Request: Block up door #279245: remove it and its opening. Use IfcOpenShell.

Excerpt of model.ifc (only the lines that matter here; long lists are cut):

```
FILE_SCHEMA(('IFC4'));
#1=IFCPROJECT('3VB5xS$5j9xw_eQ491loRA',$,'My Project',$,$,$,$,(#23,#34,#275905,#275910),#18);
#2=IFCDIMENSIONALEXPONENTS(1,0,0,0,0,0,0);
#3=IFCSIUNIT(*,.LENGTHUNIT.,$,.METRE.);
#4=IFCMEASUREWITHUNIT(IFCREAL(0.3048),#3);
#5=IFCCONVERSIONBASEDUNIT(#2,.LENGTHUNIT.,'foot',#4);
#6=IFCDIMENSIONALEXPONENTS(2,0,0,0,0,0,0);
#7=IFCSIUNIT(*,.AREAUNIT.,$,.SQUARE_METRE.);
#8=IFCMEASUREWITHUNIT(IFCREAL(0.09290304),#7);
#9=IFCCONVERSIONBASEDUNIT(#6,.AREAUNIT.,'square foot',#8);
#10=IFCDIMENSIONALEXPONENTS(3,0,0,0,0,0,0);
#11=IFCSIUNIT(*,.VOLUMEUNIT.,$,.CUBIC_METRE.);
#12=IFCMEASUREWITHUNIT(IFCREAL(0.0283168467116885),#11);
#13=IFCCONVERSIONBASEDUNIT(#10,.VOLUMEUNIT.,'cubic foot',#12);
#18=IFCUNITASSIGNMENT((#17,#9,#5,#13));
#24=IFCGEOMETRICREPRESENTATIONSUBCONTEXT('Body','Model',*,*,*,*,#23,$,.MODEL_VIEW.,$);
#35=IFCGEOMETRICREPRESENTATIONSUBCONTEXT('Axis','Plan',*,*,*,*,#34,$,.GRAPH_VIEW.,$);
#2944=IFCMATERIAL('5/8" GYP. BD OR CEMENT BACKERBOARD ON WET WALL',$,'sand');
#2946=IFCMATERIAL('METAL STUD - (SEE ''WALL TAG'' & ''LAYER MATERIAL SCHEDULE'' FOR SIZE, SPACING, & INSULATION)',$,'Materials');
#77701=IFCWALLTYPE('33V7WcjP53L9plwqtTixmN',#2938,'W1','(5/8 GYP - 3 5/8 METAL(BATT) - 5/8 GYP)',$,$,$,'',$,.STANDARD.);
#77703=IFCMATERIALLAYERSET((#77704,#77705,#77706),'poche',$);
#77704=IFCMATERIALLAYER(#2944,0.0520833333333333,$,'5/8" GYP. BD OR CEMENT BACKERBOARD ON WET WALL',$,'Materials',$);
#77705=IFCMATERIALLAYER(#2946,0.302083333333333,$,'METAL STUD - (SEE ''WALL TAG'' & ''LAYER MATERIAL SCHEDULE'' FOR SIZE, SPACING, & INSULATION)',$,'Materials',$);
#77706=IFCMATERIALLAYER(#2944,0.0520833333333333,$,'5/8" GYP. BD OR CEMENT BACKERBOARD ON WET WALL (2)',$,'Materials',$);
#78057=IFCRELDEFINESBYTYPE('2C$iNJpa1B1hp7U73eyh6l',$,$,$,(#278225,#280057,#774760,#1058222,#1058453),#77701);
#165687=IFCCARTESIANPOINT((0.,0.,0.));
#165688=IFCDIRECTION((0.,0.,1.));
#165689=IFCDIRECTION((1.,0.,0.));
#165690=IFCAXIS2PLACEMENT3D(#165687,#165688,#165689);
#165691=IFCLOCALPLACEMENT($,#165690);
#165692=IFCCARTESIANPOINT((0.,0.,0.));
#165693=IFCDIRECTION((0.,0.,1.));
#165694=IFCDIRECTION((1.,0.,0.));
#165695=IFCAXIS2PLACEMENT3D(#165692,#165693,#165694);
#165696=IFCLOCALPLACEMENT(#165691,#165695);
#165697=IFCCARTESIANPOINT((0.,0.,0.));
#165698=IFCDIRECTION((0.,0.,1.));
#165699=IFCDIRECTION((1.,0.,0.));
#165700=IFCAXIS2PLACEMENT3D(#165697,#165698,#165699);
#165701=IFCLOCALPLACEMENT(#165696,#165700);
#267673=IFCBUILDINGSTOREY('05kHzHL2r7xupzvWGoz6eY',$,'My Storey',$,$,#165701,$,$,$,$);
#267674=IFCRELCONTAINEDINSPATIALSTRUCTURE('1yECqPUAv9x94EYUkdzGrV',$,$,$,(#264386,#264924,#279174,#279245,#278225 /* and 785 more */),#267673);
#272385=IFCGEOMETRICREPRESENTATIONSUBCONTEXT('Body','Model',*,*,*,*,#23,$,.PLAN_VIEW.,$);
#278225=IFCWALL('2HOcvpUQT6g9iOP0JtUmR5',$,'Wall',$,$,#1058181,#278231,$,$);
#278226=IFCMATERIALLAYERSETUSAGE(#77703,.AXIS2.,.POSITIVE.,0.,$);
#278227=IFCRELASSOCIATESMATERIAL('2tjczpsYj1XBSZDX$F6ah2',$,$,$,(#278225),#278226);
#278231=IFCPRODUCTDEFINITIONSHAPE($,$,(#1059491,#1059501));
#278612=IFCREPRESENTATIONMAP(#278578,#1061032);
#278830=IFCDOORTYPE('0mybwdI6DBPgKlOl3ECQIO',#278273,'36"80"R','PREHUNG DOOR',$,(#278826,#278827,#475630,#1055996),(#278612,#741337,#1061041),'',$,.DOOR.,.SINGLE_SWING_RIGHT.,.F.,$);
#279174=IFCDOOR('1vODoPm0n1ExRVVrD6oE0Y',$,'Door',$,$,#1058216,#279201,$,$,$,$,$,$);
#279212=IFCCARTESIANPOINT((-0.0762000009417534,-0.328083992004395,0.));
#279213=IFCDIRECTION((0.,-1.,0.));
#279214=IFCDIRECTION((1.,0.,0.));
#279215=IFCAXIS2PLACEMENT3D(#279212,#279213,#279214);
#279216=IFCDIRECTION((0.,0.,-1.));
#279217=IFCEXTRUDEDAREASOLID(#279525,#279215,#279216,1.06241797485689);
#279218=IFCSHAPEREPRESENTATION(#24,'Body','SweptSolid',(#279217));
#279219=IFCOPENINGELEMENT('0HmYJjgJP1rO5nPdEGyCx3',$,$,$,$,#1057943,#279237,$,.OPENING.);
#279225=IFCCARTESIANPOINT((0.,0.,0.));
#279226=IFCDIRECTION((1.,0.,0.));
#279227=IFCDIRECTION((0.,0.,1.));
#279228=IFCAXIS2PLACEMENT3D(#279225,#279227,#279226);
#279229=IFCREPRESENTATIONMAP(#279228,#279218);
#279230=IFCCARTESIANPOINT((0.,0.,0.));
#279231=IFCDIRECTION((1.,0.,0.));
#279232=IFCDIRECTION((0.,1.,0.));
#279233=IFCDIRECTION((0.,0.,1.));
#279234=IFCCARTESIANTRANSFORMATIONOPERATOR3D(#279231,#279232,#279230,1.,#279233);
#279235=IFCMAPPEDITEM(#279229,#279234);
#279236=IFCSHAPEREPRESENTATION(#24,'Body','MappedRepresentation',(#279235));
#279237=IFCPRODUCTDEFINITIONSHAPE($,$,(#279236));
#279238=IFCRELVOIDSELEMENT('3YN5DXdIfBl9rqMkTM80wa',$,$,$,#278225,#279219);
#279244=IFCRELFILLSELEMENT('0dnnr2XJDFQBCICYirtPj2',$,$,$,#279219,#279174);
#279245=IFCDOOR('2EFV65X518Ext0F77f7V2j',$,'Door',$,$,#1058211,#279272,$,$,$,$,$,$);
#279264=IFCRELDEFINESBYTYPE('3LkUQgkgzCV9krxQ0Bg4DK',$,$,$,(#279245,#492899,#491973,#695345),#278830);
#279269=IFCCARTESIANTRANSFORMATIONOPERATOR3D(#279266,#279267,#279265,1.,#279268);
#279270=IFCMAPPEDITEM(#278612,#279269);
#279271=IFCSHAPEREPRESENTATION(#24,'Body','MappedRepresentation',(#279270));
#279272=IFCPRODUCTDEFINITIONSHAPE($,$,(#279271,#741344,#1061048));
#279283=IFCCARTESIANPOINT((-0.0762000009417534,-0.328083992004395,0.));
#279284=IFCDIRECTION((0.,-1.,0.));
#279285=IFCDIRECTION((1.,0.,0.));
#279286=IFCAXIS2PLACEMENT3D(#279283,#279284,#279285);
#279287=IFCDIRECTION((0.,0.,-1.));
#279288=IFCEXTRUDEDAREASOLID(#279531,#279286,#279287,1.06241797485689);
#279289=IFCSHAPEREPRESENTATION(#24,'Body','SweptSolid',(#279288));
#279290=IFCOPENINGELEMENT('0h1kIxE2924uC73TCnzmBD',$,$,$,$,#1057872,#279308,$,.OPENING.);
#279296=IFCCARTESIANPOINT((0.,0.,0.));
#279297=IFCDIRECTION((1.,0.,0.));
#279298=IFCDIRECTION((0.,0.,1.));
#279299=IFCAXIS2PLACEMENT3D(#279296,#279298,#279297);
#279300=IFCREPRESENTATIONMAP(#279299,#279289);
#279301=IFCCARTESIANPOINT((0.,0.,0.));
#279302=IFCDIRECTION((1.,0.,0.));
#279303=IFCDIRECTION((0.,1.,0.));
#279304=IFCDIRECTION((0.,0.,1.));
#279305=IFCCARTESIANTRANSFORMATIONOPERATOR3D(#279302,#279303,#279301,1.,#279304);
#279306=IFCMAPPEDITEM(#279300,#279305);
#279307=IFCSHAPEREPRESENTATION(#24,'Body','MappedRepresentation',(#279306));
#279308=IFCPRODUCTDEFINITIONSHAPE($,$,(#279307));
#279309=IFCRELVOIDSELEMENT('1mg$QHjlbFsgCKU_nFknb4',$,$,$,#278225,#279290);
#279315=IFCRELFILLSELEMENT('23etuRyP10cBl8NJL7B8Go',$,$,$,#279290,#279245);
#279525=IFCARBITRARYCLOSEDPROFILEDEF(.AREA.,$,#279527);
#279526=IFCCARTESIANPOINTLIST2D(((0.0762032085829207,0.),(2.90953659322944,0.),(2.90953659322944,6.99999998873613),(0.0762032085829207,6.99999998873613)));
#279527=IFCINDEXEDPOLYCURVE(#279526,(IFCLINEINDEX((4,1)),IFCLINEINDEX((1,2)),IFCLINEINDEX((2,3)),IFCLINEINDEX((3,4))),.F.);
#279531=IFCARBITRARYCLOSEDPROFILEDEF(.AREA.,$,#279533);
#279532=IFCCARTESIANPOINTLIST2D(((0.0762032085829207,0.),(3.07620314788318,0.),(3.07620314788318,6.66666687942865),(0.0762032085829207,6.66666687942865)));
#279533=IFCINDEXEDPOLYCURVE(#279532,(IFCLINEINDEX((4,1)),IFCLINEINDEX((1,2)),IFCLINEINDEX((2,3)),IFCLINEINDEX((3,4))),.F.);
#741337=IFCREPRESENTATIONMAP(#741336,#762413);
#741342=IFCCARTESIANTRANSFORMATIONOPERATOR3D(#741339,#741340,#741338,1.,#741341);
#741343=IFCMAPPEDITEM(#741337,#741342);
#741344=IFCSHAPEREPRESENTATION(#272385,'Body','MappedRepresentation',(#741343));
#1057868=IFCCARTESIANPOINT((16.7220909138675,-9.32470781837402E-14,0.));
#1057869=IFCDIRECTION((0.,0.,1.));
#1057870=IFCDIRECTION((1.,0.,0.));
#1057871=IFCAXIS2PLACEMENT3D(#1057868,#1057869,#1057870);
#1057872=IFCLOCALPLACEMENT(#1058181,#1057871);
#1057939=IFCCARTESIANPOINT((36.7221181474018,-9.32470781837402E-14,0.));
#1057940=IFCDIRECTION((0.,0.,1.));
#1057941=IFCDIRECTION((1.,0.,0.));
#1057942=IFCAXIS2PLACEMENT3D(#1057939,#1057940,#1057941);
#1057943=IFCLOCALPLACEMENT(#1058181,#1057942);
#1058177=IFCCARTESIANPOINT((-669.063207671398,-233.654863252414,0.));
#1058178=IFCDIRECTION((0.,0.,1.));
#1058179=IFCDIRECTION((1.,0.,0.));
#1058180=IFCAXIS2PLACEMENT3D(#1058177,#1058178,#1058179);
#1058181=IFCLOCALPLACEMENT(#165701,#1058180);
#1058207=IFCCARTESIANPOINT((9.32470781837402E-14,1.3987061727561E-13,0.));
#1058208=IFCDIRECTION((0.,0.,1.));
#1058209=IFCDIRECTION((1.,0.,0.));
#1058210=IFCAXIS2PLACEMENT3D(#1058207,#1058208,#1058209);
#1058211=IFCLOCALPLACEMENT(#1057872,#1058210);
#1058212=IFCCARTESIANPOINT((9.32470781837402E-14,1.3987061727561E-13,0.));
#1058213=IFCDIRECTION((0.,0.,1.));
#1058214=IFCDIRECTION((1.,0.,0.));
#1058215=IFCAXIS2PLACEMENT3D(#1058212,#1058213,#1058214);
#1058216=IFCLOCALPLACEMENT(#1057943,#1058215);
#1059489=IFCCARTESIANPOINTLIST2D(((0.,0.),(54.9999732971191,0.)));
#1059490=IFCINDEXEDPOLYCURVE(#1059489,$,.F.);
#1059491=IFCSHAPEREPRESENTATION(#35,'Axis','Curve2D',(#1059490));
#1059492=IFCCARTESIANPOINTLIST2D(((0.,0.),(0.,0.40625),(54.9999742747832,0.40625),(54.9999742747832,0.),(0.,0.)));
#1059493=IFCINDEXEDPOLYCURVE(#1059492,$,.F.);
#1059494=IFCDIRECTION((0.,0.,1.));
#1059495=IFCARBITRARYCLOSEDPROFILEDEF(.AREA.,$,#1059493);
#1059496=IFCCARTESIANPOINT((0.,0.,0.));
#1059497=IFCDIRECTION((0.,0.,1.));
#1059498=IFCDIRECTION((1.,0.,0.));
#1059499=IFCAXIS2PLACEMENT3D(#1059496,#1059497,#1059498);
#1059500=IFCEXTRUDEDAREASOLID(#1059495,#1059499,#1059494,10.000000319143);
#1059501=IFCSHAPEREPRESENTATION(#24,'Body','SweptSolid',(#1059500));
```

```python
import ifcopenshell
import ifcopenshell.api.feature
import ifcopenshell.api.root
import ifcopenshell.geom
import ifcopenshell.util.shape

model = ifcopenshell.open("model.ifc")
settings = ifcopenshell.geom.settings()


def volume(element):
    """Net volume in cubic metres, openings subtracted."""
    shape = ifcopenshell.geom.create_shape(settings, element)
    return ifcopenshell.util.shape.get_volume(shape.geometry)


door = model.by_id(279245)
opening = door.FillsVoids[0].RelatingOpeningElement
wall = opening.VoidsElements[0].RelatingBuildingElement
before = volume(wall)

ifcopenshell.api.root.remove_product(model, product=door)
ifcopenshell.api.feature.remove_feature(model, feature=opening)

after = volume(wall)

print(f"wall volume {before:.3f} -> {after:.3f} m3")

model.write("model-out.ifc")
```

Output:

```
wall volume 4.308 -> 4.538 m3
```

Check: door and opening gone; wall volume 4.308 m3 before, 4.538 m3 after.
